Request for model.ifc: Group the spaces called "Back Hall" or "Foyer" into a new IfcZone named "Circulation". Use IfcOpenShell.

First a look at what the model holds.

```python
import ifcopenshell

model = ifcopenshell.open("model.ifc")
print(model.schema)
seen = {}
for space in model.by_type("IfcSpace"):
    seen[space.LongName] = seen.get(space.LongName, 0) + 1
for name, count in sorted(seen.items(), key=str):
    print(count, "x", name)
print("zones:", [z.Name for z in model.by_type("IfcZone")][:20])
```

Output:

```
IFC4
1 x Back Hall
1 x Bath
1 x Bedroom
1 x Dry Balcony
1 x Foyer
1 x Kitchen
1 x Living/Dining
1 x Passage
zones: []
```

```python
import ifcopenshell
import ifcopenshell.api.group
import ifcopenshell.api.root

model = ifcopenshell.open("model.ifc")

names = {"Back Hall", "Foyer"}
spaces = [s for s in model.by_type("IfcSpace") if s.LongName in names]

zone = ifcopenshell.api.root.create_entity(model, ifc_class="IfcZone", name="Circulation")
ifcopenshell.api.group.assign_group(model, products=spaces, group=zone)
print(len(spaces), "spaces in", zone.Name)

model.write("model_v2.ifc")
```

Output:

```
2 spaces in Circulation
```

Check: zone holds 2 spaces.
